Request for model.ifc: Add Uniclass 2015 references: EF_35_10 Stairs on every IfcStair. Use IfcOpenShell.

First a look at what the model holds.

```python
import ifcopenshell

model = ifcopenshell.open("model.ifc")
print(model.schema)
print("classifications:", [c.Name for c in model.by_type("IfcClassification")])
for ifc_class in ("IfcDoor", "IfcRoof", "IfcStair", "IfcWall", "IfcWindow"):
    print(ifc_class, len(model.by_type(ifc_class)))
```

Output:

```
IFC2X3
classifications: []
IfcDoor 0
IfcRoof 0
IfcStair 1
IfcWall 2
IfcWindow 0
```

```python
import ifcopenshell
import ifcopenshell.api.classification

model = ifcopenshell.open("model.ifc")

# IFC2X3 requires Source and Edition and has no link from the project to the system.
system = model.create_entity("IfcClassification", Source="NBS", Edition="2015", Name="Uniclass 2015")

codes = {
    "IfcStair": ("EF_35_10", "Stairs"),
}
for ifc_class, (code, name) in codes.items():
    products = model.by_type(ifc_class)
    ifcopenshell.api.classification.add_reference(
        model, products=products, classification=system, identification=code, name=name
    )
    print(code, len(products))

model.write("model_updated.ifc")
```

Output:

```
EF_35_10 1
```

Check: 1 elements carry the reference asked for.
